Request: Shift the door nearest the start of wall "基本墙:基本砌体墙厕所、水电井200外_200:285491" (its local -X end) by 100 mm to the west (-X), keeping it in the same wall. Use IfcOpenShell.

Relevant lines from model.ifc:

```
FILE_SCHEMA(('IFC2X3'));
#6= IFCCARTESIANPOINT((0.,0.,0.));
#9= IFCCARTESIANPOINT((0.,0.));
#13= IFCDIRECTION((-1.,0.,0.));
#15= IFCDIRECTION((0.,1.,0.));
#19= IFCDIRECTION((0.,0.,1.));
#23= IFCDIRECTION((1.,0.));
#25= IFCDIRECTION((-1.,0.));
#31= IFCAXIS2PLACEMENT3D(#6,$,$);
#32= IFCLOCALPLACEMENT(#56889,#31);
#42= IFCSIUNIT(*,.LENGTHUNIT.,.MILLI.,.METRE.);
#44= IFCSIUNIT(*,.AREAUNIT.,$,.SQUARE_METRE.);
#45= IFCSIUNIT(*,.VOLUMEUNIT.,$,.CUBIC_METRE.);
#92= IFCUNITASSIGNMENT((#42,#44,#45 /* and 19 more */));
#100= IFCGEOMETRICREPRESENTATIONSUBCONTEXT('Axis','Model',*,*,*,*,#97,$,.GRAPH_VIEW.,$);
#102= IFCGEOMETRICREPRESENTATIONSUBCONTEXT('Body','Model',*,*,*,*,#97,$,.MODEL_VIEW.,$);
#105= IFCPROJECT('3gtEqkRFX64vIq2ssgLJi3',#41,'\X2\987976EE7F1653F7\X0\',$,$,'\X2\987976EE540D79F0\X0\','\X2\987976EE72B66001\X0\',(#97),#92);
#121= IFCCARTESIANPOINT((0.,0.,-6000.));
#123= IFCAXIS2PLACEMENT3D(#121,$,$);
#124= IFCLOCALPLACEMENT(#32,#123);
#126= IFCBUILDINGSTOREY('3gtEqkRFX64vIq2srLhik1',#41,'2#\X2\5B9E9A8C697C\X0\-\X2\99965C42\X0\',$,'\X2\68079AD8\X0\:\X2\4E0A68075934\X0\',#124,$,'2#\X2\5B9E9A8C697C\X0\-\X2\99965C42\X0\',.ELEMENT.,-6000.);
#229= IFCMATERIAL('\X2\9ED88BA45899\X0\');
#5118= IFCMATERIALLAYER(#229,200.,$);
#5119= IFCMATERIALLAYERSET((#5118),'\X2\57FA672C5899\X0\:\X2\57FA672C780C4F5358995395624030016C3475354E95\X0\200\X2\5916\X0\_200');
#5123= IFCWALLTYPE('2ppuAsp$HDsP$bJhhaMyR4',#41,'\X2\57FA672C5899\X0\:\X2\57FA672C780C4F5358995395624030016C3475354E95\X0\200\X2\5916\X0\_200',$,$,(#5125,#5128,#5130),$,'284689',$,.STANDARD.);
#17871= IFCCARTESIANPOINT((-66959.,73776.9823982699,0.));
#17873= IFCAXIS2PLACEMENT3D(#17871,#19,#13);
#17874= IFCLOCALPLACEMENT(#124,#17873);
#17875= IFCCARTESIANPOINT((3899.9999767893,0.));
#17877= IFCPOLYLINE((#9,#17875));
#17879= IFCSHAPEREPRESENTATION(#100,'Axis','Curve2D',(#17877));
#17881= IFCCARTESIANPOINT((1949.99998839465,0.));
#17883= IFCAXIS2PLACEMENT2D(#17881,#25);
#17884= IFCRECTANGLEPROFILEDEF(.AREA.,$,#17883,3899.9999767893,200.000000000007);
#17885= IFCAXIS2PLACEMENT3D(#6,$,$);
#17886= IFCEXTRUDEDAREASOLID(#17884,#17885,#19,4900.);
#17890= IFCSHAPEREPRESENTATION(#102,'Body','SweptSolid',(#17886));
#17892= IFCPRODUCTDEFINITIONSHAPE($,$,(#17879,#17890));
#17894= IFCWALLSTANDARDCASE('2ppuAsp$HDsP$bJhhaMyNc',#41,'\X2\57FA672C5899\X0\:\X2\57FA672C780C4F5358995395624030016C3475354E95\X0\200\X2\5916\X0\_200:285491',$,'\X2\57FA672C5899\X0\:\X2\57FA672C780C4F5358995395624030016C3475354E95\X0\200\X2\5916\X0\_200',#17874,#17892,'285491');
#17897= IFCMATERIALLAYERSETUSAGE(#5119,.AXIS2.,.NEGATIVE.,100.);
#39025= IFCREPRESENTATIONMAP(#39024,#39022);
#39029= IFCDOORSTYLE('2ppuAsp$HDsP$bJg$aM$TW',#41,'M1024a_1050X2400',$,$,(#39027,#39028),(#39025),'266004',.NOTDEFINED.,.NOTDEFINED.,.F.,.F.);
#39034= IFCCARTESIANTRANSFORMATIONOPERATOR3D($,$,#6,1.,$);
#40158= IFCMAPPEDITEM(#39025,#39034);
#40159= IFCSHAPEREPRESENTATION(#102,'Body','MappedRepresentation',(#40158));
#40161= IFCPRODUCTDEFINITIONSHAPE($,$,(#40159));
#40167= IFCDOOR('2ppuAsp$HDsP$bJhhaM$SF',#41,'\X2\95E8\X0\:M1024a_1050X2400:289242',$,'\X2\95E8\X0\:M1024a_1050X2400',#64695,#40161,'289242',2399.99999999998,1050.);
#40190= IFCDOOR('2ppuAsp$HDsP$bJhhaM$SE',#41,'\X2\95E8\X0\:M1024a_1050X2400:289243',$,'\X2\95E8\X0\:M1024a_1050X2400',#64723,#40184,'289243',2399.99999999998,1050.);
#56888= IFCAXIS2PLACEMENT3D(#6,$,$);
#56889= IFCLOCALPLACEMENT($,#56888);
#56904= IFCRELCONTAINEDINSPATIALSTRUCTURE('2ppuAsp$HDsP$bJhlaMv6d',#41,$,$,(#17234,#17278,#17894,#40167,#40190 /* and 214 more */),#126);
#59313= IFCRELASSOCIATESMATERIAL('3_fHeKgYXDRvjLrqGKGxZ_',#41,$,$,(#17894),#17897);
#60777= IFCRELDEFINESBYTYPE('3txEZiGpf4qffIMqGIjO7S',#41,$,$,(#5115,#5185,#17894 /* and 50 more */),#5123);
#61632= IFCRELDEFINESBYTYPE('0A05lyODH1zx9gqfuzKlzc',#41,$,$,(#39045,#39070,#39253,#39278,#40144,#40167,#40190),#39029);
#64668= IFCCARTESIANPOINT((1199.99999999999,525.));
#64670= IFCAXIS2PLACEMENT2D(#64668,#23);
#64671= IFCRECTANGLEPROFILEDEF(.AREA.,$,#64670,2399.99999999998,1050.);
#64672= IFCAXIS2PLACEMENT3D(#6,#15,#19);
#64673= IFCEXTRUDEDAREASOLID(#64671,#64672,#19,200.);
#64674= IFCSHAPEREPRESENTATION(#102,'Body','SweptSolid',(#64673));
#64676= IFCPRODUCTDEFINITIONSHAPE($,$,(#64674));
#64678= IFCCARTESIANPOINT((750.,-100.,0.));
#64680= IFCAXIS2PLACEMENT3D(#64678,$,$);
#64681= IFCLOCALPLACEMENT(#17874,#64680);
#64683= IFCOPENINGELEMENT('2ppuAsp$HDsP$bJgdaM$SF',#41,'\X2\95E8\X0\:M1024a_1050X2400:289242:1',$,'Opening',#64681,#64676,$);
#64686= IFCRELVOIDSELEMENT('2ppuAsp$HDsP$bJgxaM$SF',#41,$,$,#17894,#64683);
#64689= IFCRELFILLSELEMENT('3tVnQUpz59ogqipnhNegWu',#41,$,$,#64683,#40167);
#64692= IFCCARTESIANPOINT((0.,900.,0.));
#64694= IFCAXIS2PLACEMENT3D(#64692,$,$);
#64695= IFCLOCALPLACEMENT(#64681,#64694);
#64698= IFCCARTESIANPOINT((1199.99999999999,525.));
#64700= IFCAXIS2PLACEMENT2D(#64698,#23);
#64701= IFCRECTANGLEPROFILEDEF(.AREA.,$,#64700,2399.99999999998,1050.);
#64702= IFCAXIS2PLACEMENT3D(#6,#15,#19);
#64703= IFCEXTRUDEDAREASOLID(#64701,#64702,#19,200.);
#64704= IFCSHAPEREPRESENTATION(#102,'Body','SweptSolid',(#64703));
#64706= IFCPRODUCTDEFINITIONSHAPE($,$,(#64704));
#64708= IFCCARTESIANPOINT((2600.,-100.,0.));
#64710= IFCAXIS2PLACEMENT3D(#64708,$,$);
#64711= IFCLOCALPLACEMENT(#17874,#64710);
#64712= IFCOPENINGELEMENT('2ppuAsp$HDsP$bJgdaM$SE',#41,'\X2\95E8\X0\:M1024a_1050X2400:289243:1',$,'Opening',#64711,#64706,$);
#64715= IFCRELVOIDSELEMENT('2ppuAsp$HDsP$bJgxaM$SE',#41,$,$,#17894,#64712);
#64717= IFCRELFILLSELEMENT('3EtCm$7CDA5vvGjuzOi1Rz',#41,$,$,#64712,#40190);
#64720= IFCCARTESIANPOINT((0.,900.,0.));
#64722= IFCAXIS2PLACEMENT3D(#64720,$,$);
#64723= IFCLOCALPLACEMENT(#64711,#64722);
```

```python
import ifcopenshell
import ifcopenshell.api.geometry
import ifcopenshell.util.placement
import ifcopenshell.util.unit

model = ifcopenshell.open("model.ifc")
unit_scale = ifcopenshell.util.unit.calculate_unit_scale(model)

door = model.by_guid("2ppuAsp$HDsP$bJhhaM$SF")
opening = door.FillsVoids[0].RelatingOpeningElement
wall = opening.VoidsElements[0].RelatingBuildingElement

wall_matrix = ifcopenshell.util.placement.get_local_placement(wall.ObjectPlacement)
shift = wall_matrix[:3, 0] * 0.1 / unit_scale
before = ifcopenshell.util.placement.get_local_placement(door.ObjectPlacement)[:3, 3].copy()

# The door is placed relative to its opening, so it follows when the opening moves.
matrix = ifcopenshell.util.placement.get_local_placement(opening.ObjectPlacement)
matrix[:3, 3] += shift
ifcopenshell.api.geometry.edit_object_placement(
    model, product=opening, matrix=matrix, is_si=False, should_transform_children=True
)

after = ifcopenshell.util.placement.get_local_placement(door.ObjectPlacement)[:3, 3]
print("door moved by", (after - before).round(3) + 0.0)

model.write("model_rev.ifc")
```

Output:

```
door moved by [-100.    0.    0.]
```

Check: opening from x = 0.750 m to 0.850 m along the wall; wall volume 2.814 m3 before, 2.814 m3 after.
